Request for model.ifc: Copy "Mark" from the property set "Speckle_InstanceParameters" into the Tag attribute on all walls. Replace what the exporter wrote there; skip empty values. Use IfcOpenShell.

First a look at what the model holds.

```python
import ifcopenshell
import ifcopenshell.util.element

model = ifcopenshell.open("model.ifc")
print(model.schema)
walls = model.by_type("IfcWall")
print(len(walls), "walls")
for e in walls[:8]:
    source = ifcopenshell.util.element.get_pset(e, "Speckle_InstanceParameters", "Mark")
    target = e.Tag
    print(e.id(), repr(source), repr(target), sep=" | ")
```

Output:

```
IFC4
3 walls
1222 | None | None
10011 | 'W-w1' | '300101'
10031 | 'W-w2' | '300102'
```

```python
import ifcopenshell
import ifcopenshell.util.element

model = ifcopenshell.open("model.ifc")

count = 0
for e in model.by_type("IfcWall"):
    value = ifcopenshell.util.element.get_pset(e, "Speckle_InstanceParameters", "Mark")
    current = e.Tag
    if not value or not value.strip() or current == value:
        continue
    e.Tag = value
    count += 1

print(count, "walls updated")

model.write("model-out.ifc")
```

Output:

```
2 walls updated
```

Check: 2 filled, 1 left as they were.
